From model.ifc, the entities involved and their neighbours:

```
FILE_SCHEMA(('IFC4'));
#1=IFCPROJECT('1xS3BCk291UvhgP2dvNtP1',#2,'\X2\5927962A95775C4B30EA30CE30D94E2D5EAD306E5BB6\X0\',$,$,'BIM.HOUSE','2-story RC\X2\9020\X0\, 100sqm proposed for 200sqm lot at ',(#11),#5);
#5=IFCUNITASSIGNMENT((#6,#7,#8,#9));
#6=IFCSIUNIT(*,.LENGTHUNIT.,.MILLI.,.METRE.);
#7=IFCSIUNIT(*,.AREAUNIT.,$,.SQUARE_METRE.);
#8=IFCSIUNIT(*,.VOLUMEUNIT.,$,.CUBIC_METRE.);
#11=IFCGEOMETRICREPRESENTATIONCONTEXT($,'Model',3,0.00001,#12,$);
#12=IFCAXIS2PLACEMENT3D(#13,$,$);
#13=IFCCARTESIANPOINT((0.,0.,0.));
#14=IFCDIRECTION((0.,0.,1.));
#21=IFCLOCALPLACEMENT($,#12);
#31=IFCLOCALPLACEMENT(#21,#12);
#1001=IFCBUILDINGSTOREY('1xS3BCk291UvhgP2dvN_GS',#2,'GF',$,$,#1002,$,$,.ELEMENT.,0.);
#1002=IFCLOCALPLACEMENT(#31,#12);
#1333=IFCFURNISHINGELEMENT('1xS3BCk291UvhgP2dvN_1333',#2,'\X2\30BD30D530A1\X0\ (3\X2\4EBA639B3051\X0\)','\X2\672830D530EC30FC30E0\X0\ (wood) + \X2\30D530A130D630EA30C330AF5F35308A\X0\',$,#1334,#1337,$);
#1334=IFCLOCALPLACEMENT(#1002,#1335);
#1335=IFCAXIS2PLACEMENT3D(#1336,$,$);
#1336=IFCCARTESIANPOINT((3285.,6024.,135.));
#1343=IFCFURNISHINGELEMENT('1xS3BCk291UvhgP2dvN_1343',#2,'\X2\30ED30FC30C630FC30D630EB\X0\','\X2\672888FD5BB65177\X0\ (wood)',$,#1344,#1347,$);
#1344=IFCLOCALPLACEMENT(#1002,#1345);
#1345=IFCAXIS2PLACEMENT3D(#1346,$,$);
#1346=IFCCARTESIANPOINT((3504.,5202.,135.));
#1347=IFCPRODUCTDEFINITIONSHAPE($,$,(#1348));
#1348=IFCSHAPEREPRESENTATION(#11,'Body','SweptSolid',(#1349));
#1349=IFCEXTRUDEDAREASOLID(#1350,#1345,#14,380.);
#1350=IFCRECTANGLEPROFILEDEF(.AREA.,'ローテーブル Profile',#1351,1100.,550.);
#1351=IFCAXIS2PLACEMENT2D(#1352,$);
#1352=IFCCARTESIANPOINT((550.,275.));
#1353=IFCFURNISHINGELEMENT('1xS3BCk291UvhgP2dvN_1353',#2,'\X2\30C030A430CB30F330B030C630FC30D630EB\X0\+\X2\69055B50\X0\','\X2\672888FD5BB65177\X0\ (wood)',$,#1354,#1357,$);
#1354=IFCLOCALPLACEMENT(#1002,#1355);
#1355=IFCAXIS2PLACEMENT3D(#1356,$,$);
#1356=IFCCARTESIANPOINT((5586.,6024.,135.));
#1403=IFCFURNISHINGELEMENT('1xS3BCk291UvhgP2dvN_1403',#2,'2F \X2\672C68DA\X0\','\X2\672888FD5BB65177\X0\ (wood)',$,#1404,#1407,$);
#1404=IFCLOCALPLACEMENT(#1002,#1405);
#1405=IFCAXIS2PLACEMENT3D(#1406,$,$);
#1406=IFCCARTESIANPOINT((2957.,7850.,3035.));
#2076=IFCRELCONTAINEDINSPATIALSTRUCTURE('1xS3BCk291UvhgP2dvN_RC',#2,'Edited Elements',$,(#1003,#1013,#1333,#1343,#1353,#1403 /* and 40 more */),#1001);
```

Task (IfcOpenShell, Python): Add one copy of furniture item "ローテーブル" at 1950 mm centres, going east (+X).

```python
import numpy as np
import ifcopenshell
import ifcopenshell.api.geometry
import ifcopenshell.api.root
import ifcopenshell.util.element
import ifcopenshell.util.placement
import ifcopenshell.util.unit

model = ifcopenshell.open("model.ifc")
unit_scale = ifcopenshell.util.unit.calculate_unit_scale(model)


def reuse_history(source, copy):
    """copy_class also copies each property set's owner history, people and application; keep the originals."""
    for rel in copy.IsDefinedBy:
        if rel.is_a("IfcRelDefinesByProperties") and (history := rel.RelatingPropertyDefinition.OwnerHistory):
            rel.RelatingPropertyDefinition.OwnerHistory = source.OwnerHistory
            ifcopenshell.util.element.remove_deep2(model, history)


source = model.by_guid("1xS3BCk291UvhgP2dvN_1343")
base = ifcopenshell.util.placement.get_local_placement(source.ObjectPlacement)
step = np.array([1.0, 0.0, 0.0]) * 1.95 / unit_scale

for i in range(1, 2):
    copy = ifcopenshell.api.root.copy_class(model, product=source)
    copy.Representation = ifcopenshell.util.element.copy_deep(
        model, source.Representation, exclude=["IfcGeometricRepresentationContext", "IfcRepresentationMap"]
    )
    reuse_history(source, copy)
    matrix = base.copy()
    matrix[:3, 3] += i * step
    print("added at", matrix[:3, 3].round(3) + 0.0)
    ifcopenshell.api.geometry.edit_object_placement(model, product=copy, matrix=matrix, is_si=False)

model.write("model-out.ifc")
```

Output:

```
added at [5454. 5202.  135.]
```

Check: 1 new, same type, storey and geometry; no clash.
